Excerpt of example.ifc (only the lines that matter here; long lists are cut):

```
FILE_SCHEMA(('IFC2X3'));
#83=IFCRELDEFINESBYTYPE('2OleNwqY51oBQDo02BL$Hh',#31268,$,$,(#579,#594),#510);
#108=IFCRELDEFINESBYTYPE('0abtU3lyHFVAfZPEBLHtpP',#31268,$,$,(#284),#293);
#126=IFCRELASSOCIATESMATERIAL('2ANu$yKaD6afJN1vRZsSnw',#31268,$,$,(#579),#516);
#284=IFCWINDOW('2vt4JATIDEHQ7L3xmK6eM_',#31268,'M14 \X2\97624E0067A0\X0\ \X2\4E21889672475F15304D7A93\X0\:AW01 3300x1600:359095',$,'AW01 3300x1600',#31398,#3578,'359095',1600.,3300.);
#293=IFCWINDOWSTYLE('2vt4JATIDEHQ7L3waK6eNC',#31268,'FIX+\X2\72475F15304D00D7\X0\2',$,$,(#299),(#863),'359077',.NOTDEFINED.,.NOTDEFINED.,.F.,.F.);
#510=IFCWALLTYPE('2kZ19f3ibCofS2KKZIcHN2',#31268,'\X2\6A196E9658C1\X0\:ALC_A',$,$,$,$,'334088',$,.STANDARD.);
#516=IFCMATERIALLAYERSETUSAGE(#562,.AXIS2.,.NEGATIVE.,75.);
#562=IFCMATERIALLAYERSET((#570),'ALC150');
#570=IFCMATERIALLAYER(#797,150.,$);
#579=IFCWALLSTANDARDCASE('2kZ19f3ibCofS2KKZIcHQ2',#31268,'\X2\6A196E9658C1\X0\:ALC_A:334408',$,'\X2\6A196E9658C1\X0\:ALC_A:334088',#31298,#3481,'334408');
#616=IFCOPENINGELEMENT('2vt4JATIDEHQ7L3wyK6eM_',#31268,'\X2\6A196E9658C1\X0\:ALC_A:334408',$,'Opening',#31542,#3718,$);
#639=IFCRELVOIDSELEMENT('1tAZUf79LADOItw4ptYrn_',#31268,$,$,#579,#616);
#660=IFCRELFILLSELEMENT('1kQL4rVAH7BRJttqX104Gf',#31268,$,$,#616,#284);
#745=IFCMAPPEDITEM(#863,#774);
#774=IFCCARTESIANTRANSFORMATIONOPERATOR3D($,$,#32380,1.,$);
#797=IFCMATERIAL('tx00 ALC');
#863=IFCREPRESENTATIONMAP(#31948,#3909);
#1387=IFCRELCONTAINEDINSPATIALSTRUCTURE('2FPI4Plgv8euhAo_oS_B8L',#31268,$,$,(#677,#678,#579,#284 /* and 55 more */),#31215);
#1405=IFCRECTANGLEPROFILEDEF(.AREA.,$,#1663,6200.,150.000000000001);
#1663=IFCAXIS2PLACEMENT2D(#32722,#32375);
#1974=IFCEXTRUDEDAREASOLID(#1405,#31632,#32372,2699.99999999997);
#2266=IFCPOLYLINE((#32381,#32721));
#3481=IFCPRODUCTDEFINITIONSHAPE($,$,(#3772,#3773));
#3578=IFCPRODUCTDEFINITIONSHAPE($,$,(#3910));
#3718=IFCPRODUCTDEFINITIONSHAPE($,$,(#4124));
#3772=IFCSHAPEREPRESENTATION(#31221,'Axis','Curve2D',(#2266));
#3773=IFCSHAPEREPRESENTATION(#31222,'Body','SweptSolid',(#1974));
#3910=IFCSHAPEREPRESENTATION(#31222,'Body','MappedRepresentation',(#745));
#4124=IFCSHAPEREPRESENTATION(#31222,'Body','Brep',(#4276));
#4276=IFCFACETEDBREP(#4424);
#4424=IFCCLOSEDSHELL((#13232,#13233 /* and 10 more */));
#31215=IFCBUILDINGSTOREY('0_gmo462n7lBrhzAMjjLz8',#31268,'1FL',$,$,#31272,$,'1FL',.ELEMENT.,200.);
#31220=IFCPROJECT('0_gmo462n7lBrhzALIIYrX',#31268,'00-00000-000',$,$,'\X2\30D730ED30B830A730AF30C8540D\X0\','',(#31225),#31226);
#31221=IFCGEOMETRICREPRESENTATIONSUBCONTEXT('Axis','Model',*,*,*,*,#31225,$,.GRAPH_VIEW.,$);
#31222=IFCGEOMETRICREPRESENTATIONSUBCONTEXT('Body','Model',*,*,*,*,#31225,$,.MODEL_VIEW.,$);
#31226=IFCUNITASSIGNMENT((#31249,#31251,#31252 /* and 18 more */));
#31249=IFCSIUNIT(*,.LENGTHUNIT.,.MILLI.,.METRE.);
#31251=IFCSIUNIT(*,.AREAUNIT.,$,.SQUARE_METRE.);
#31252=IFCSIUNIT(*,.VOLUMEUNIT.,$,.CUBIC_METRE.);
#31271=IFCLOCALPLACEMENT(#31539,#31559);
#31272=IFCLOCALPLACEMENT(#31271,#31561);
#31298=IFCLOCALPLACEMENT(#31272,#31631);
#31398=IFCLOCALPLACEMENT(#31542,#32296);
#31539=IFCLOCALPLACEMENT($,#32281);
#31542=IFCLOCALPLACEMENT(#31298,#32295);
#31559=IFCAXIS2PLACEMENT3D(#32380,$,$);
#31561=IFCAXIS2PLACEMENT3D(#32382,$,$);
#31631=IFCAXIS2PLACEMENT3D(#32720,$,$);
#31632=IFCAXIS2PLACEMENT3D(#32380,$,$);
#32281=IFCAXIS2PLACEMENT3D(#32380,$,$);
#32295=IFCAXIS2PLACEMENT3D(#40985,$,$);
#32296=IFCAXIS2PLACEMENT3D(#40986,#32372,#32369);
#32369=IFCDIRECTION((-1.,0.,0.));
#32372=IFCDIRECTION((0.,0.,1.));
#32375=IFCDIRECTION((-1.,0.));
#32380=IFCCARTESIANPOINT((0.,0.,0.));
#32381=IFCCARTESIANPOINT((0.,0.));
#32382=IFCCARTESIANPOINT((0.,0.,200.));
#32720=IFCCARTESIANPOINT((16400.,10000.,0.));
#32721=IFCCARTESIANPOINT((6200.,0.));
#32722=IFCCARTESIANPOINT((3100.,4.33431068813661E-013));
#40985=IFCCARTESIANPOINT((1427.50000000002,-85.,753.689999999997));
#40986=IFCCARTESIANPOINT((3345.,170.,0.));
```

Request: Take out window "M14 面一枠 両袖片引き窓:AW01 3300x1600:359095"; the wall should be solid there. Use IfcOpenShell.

```python
import ifcopenshell
import ifcopenshell.api.feature
import ifcopenshell.api.root
import ifcopenshell.geom
import ifcopenshell.util.shape

model = ifcopenshell.open("example.ifc")
settings = ifcopenshell.geom.settings()


def volume(element):
    """Net volume in cubic metres, openings subtracted."""
    shape = ifcopenshell.geom.create_shape(settings, element)
    return ifcopenshell.util.shape.get_volume(shape.geometry)


window = model.by_guid("2vt4JATIDEHQ7L3xmK6eM_")
opening = window.FillsVoids[0].RelatingOpeningElement
wall = opening.VoidsElements[0].RelatingBuildingElement
before = volume(wall)

ifcopenshell.api.root.remove_product(model, product=window)
ifcopenshell.api.feature.remove_feature(model, feature=opening)

after = volume(wall)

print(f"wall volume {before:.3f} -> {after:.3f} m3")

model.write("example_updated.ifc")
```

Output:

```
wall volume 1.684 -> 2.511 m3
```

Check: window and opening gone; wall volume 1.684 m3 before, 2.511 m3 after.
